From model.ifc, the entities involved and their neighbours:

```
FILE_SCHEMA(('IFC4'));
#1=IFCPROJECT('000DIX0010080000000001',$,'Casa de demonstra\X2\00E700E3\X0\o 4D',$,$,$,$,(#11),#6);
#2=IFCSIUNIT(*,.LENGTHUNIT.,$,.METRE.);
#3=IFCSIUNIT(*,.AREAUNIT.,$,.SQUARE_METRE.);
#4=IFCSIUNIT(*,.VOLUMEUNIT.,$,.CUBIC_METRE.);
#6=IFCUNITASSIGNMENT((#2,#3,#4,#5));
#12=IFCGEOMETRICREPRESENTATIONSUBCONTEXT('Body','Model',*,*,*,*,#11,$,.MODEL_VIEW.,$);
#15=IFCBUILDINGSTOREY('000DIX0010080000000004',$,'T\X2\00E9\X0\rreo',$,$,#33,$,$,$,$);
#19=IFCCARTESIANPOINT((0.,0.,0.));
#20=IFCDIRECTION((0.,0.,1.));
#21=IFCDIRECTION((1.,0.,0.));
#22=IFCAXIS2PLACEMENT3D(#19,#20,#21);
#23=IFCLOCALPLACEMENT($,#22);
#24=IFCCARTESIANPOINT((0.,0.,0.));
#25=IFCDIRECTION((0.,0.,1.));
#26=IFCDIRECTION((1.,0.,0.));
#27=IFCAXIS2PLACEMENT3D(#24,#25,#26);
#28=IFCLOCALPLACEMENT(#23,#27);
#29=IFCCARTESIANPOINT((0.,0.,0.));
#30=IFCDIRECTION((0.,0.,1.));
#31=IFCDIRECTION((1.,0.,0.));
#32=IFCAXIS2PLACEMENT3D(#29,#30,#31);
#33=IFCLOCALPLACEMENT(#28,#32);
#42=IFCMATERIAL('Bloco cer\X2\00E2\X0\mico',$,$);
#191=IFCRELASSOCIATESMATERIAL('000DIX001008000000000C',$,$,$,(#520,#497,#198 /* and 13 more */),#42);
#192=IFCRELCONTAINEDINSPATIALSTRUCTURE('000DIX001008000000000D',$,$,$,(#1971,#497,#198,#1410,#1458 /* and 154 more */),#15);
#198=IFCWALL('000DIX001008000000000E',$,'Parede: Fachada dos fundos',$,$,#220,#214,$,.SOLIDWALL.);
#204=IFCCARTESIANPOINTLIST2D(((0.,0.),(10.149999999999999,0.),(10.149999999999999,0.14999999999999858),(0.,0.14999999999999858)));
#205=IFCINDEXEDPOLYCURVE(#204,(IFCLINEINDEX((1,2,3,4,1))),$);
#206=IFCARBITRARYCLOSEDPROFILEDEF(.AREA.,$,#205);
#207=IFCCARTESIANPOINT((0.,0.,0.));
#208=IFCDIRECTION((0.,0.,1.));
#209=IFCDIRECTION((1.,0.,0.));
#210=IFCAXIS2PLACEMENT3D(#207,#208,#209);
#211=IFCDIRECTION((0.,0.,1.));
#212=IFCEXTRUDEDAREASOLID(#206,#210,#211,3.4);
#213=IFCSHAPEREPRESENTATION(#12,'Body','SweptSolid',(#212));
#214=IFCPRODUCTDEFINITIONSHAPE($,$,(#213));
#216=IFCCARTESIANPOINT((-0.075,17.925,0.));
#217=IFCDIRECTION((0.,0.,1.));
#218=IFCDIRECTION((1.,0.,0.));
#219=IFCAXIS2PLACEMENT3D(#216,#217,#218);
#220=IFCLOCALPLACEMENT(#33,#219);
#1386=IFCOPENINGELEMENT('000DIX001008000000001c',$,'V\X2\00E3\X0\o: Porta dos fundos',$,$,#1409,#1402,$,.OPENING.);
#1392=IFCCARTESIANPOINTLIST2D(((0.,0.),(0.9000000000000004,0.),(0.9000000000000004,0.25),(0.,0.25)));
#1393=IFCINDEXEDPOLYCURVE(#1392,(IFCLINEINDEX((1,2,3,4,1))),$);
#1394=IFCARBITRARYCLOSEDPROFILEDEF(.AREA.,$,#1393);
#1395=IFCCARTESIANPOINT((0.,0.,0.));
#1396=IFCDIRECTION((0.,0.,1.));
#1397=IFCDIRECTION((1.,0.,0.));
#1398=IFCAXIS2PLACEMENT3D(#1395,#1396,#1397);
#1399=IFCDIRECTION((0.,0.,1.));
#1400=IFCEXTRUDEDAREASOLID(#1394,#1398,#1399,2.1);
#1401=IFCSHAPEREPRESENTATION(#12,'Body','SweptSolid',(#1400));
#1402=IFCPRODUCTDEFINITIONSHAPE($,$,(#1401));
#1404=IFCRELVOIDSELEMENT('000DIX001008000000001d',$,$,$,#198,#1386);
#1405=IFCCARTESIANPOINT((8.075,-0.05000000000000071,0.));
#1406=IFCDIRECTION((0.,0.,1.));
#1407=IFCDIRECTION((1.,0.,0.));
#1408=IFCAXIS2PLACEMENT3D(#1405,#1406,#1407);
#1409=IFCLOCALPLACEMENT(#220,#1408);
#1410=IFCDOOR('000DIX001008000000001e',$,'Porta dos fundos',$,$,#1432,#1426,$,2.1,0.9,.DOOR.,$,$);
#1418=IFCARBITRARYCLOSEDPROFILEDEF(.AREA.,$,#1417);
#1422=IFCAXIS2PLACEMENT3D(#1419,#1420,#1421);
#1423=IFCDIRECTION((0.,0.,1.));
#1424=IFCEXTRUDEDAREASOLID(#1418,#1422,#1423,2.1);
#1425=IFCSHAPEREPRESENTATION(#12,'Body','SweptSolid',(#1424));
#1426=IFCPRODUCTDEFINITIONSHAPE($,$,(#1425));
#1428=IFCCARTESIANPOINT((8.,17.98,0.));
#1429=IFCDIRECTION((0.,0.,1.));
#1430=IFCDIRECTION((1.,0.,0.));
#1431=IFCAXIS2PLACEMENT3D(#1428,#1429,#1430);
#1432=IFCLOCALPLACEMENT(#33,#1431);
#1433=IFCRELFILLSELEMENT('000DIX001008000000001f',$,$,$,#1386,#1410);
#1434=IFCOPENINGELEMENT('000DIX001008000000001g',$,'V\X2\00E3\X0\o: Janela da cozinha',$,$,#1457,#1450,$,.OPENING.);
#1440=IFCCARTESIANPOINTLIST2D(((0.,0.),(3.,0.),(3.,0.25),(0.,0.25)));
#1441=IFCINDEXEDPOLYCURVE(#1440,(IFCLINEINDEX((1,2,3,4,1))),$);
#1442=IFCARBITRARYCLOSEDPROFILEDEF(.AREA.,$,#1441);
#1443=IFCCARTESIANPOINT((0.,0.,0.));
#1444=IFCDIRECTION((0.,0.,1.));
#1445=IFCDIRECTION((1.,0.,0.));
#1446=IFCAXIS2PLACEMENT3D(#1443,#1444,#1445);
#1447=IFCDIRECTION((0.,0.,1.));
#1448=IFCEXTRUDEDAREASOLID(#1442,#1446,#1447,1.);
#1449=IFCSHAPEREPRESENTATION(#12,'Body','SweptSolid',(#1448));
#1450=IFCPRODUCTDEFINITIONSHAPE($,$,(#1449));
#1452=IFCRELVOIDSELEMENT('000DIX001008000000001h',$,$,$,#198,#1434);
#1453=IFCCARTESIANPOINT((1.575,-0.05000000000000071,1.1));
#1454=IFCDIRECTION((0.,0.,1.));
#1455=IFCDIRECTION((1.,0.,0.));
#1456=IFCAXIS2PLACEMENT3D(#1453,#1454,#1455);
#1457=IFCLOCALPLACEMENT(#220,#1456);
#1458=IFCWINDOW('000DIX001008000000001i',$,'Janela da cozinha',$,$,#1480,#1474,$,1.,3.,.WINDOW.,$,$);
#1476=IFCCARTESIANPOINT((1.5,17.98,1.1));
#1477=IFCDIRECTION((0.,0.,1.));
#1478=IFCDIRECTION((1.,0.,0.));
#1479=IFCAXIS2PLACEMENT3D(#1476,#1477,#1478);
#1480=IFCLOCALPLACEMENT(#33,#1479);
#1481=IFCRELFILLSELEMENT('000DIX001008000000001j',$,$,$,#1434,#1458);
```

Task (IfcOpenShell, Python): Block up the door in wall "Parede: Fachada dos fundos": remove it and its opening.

```python
import ifcopenshell
import ifcopenshell.api.feature
import ifcopenshell.api.root
import ifcopenshell.geom
import ifcopenshell.util.shape

model = ifcopenshell.open("model.ifc")
settings = ifcopenshell.geom.settings()


def volume(element):
    """Net volume in cubic metres, openings subtracted."""
    shape = ifcopenshell.geom.create_shape(settings, element)
    return ifcopenshell.util.shape.get_volume(shape.geometry)


door = model.by_guid("000DIX001008000000001e")
opening = door.FillsVoids[0].RelatingOpeningElement
wall = opening.VoidsElements[0].RelatingBuildingElement
before = volume(wall)

ifcopenshell.api.root.remove_product(model, product=door)
ifcopenshell.api.feature.remove_feature(model, feature=opening)

after = volume(wall)

print(f"wall volume {before:.3f} -> {after:.3f} m3")

model.write("model-out.ifc")
```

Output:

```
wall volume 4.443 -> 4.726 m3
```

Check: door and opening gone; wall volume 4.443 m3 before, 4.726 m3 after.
